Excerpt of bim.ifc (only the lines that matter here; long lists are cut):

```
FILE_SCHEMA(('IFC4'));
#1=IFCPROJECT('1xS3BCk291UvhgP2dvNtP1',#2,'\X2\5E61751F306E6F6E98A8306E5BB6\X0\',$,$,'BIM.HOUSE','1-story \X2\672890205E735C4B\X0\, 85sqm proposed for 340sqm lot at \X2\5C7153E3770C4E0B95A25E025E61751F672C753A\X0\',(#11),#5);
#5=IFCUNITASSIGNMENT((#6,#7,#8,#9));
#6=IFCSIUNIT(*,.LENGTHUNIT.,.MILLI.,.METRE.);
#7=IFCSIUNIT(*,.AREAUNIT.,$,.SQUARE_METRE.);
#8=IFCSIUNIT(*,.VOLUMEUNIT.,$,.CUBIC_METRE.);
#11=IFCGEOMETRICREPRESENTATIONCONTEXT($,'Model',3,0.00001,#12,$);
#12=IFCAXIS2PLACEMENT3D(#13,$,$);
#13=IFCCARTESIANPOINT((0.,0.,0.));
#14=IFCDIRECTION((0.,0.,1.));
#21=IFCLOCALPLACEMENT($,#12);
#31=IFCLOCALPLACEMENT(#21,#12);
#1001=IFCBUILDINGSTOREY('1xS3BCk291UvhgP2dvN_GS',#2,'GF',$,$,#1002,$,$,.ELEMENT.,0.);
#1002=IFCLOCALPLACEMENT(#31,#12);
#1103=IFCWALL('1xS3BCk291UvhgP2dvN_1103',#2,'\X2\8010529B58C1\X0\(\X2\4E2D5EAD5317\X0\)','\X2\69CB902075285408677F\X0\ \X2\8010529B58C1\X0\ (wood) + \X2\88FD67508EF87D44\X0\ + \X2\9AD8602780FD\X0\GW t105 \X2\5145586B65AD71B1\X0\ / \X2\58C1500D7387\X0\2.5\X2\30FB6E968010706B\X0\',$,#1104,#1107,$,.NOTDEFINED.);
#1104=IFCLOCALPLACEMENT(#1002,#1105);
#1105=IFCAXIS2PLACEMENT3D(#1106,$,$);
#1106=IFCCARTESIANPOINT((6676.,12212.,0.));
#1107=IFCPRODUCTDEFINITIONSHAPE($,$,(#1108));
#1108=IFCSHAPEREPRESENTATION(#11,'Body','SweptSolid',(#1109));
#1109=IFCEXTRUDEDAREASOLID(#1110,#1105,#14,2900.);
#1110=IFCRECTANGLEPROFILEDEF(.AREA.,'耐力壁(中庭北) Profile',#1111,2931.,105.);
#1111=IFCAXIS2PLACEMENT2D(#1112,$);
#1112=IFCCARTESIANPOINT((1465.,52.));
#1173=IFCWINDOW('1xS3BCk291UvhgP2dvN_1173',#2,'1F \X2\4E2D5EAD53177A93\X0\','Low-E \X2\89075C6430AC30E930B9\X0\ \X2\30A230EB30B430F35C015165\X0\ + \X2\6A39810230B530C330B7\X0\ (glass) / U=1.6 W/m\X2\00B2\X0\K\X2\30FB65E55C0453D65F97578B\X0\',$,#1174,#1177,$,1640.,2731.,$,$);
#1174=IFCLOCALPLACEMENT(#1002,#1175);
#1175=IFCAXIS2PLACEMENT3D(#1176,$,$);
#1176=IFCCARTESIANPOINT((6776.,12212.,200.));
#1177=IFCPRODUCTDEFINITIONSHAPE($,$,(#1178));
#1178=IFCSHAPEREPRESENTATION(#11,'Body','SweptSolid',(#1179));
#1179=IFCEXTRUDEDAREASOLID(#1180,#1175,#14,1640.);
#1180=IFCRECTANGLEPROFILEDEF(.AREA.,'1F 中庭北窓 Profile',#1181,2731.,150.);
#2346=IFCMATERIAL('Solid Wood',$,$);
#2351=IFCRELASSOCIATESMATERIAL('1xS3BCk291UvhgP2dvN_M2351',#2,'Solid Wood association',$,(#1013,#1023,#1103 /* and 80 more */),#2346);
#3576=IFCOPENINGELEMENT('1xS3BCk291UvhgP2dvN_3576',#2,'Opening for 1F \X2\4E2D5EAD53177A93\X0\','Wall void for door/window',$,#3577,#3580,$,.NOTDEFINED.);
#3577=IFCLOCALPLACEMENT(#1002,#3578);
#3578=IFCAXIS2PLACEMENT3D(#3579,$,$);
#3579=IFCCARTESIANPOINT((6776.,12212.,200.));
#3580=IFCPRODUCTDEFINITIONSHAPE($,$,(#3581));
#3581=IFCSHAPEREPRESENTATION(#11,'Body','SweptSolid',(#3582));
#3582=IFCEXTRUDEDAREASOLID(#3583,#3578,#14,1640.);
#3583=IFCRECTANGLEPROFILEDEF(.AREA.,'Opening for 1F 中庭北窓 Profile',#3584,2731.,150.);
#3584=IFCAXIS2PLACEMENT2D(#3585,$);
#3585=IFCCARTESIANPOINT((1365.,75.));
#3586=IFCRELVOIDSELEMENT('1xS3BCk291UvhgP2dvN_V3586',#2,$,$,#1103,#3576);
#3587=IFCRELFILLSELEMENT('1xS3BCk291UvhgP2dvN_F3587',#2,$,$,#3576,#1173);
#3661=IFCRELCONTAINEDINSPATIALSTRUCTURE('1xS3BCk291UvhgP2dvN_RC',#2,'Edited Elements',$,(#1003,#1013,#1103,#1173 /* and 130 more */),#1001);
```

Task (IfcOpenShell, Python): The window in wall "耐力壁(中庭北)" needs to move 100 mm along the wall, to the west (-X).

```python
import ifcopenshell
import ifcopenshell.api.geometry
import ifcopenshell.util.placement
import ifcopenshell.util.unit

model = ifcopenshell.open("bim.ifc")
unit_scale = ifcopenshell.util.unit.calculate_unit_scale(model)

window = model.by_id(1173)
opening = window.FillsVoids[0].RelatingOpeningElement
wall = opening.VoidsElements[0].RelatingBuildingElement

wall_matrix = ifcopenshell.util.placement.get_local_placement(wall.ObjectPlacement)
shift = wall_matrix[:3, 0] * -0.1 / unit_scale
before = ifcopenshell.util.placement.get_local_placement(window.ObjectPlacement)[:3, 3].copy()

# The window is not placed relative to its opening, so move both.
for product in (opening, window):
    matrix = ifcopenshell.util.placement.get_local_placement(product.ObjectPlacement)
    matrix[:3, 3] += shift
    ifcopenshell.api.geometry.edit_object_placement(model, product=product, matrix=matrix, is_si=False)

after = ifcopenshell.util.placement.get_local_placement(window.ObjectPlacement)[:3, 3]
print("window moved by", (after - before).round(3) + 0.0)

model.write("bim_v2.ifc")
```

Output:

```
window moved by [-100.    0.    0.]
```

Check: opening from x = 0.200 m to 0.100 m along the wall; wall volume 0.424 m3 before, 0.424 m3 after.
